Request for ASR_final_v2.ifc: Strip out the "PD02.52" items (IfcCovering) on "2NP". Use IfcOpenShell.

First a look at what the model holds.

```python
import ifcopenshell
import ifcopenshell.util.element

model = ifcopenshell.open("ASR_final_v2.ifc")
print(model.schema)
storey = next(s for s in model.by_type("IfcBuildingStorey") if s.Name == "2NP")
coverings = [e for e in ifcopenshell.util.element.get_decomposition(storey) if e.is_a("IfcCovering")]
seen = {}
for e in coverings:
    element_type = ifcopenshell.util.element.get_type(e)
    name = element_type.Name if element_type not in (None, e) else None
    seen[name] = seen.get(name, 0) + 1
for name, count in sorted(seen.items(), key=str):
    print(count, "x", name)
```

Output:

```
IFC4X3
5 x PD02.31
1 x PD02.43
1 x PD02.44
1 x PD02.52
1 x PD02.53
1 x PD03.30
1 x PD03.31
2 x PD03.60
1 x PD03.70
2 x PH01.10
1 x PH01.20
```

```python
import ifcopenshell
import ifcopenshell.api.root
import ifcopenshell.util.element

model = ifcopenshell.open("ASR_final_v2.ifc")

storey = next(s for s in model.by_type("IfcBuildingStorey") if s.Name == "2NP")
coverings = [e for e in ifcopenshell.util.element.get_decomposition(storey) if e.is_a("IfcCovering")]
targets = [e for e in coverings if (t := ifcopenshell.util.element.get_type(e)) not in (None, e) and t.Name == "PD02.52"]

for e in targets:
    ifcopenshell.api.root.remove_product(model, product=e)
print(len(targets), "removed")

model.write("ASR_final_v2_updated.ifc")
```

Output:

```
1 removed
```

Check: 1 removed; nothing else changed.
